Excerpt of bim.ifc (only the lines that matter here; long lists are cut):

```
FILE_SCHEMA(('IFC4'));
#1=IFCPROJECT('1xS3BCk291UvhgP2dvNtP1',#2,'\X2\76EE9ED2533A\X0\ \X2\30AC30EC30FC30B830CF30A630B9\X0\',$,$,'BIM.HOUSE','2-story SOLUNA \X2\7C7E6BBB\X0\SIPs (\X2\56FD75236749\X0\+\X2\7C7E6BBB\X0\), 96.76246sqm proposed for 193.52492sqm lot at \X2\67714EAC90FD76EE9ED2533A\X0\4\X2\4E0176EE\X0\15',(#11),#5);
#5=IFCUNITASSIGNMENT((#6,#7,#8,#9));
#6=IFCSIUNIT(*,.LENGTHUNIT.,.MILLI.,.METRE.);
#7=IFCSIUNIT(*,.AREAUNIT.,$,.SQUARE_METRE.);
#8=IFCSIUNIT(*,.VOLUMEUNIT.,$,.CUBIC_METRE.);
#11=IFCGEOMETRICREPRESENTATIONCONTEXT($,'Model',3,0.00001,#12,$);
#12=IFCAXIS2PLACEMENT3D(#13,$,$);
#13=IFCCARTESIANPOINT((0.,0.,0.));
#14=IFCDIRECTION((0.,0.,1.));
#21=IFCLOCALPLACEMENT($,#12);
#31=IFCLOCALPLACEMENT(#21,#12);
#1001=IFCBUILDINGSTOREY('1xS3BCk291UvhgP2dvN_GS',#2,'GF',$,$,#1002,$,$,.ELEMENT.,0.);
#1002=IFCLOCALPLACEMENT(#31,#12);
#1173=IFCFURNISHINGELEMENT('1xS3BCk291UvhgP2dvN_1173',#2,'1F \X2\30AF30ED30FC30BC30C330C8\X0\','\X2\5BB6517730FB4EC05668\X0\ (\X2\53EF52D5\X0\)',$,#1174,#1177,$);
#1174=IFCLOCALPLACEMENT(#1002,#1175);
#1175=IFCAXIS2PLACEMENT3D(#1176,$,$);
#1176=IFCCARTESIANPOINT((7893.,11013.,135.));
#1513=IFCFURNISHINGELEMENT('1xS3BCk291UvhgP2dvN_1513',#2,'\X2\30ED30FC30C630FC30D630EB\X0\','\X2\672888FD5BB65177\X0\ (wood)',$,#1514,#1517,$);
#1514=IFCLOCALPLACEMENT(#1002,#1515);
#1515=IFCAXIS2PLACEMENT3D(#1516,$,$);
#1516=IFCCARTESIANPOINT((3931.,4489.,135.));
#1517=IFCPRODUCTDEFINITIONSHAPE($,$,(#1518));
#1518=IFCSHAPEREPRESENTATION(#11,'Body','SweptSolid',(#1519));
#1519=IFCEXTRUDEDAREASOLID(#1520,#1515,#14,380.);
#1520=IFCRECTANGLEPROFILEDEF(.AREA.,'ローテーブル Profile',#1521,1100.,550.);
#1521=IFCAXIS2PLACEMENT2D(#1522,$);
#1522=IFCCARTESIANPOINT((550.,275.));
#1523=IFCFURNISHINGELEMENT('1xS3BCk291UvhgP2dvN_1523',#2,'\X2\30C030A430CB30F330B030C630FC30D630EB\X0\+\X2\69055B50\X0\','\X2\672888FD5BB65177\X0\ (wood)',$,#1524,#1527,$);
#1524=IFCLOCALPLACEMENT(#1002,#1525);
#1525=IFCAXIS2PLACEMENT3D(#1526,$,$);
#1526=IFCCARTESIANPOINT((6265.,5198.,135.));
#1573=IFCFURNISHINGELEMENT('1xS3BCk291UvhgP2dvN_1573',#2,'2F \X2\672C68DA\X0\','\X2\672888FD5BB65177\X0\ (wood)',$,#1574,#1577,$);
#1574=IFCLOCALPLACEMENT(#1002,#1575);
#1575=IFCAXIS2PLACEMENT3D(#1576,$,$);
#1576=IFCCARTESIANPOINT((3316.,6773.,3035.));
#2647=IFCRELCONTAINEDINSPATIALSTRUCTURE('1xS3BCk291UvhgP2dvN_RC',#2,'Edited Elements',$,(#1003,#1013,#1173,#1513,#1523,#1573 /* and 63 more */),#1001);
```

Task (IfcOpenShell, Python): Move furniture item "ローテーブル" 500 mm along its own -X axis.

```python
import ifcopenshell
import ifcopenshell.api.geometry
import ifcopenshell.util.placement
import ifcopenshell.util.unit

model = ifcopenshell.open("bim.ifc")
unit_scale = ifcopenshell.util.unit.calculate_unit_scale(model)

item = model.by_guid("1xS3BCk291UvhgP2dvN_1513")
matrix = ifcopenshell.util.placement.get_local_placement(item.ObjectPlacement)
matrix[:3, 3] -= matrix[:3, 0] * 0.5 / unit_scale
ifcopenshell.api.geometry.edit_object_placement(model, product=item, matrix=matrix, is_si=False)

print(ifcopenshell.util.placement.get_local_placement(item.ObjectPlacement).round(3) + 0.0)

model.write("bim_v2.ifc")
```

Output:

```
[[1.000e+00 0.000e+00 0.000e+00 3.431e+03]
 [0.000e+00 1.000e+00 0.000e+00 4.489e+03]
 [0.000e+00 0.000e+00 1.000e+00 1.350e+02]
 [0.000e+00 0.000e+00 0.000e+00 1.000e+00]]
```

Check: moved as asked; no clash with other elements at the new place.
